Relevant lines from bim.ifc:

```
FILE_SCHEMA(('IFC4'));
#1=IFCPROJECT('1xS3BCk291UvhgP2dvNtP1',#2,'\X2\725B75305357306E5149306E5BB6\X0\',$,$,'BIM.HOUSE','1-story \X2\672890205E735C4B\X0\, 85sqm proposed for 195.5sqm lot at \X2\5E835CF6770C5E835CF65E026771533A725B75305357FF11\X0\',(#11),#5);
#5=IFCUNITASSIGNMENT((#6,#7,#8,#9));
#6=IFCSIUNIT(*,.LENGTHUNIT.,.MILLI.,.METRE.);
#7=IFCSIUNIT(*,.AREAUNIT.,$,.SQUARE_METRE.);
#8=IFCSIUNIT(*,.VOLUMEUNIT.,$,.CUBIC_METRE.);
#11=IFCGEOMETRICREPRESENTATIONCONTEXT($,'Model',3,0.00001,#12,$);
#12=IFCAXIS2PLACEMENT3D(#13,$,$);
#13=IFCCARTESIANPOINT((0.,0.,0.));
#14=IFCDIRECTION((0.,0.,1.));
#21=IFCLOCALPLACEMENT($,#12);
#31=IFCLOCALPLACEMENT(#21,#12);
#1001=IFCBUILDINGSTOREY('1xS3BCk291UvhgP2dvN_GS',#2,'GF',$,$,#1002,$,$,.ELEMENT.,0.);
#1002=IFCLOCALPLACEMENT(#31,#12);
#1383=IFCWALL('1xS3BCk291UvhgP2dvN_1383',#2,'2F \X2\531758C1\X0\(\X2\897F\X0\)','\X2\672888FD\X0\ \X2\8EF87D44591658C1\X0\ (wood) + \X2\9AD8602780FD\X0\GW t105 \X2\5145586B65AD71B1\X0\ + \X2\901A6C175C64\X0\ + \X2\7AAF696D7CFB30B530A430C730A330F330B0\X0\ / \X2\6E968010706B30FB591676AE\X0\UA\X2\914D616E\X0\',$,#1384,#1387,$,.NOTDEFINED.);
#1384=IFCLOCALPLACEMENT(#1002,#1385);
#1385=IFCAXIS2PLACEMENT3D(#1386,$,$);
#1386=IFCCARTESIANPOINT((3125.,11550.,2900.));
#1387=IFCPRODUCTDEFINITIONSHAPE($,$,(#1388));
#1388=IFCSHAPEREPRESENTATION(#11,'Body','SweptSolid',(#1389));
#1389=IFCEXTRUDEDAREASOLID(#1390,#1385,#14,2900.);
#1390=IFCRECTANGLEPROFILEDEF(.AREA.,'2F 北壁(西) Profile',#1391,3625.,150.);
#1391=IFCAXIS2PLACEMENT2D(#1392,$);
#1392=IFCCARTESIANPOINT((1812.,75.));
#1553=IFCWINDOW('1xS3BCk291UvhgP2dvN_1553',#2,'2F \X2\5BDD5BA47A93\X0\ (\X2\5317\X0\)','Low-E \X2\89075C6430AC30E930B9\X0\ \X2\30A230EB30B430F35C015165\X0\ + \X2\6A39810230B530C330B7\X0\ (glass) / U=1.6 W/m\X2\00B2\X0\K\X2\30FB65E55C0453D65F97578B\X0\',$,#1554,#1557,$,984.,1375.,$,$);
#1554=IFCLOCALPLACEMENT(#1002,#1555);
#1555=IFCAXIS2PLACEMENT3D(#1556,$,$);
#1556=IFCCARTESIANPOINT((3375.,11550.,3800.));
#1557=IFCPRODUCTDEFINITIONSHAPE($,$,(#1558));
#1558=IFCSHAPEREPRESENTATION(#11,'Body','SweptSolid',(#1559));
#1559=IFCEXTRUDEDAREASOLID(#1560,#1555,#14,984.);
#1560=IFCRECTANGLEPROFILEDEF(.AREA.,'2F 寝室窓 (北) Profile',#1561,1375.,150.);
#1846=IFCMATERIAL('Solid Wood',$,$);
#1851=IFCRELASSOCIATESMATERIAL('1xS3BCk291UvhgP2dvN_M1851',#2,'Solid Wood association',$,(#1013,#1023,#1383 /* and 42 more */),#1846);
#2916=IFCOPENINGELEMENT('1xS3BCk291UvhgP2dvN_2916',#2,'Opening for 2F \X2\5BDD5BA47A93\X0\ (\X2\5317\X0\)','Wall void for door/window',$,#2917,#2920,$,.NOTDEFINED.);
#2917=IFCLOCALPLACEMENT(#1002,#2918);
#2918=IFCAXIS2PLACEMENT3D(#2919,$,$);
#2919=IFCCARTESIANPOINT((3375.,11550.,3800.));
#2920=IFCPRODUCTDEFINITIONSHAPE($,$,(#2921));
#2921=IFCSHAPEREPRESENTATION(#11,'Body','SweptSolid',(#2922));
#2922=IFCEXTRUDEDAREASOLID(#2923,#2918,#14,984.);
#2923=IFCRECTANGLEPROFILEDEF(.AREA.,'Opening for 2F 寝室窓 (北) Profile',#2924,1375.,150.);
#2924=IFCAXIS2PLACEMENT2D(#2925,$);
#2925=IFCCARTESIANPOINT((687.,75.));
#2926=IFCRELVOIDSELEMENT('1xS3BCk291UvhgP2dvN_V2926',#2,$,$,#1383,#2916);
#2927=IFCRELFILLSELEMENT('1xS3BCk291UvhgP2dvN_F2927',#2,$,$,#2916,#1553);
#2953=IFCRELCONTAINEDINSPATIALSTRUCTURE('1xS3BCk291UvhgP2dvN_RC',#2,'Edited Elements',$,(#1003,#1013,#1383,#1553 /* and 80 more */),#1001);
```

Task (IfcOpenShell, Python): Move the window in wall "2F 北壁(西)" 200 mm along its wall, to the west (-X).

```python
import ifcopenshell
import ifcopenshell.api.geometry
import ifcopenshell.util.placement
import ifcopenshell.util.unit

model = ifcopenshell.open("bim.ifc")
unit_scale = ifcopenshell.util.unit.calculate_unit_scale(model)

window = model.by_guid("1xS3BCk291UvhgP2dvN_1553")
opening = window.FillsVoids[0].RelatingOpeningElement
wall = opening.VoidsElements[0].RelatingBuildingElement

wall_matrix = ifcopenshell.util.placement.get_local_placement(wall.ObjectPlacement)
shift = wall_matrix[:3, 0] * -0.2 / unit_scale
before = ifcopenshell.util.placement.get_local_placement(window.ObjectPlacement)[:3, 3].copy()

# The window is not placed relative to its opening, so move both.
for product in (opening, window):
    matrix = ifcopenshell.util.placement.get_local_placement(product.ObjectPlacement)
    matrix[:3, 3] += shift
    ifcopenshell.api.geometry.edit_object_placement(model, product=product, matrix=matrix, is_si=False)

after = ifcopenshell.util.placement.get_local_placement(window.ObjectPlacement)[:3, 3]
print("window moved by", (after - before).round(3) + 0.0)

model.write("bim_rev.ifc")
```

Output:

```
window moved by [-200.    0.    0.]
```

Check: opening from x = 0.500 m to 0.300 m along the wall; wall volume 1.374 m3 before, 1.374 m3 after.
